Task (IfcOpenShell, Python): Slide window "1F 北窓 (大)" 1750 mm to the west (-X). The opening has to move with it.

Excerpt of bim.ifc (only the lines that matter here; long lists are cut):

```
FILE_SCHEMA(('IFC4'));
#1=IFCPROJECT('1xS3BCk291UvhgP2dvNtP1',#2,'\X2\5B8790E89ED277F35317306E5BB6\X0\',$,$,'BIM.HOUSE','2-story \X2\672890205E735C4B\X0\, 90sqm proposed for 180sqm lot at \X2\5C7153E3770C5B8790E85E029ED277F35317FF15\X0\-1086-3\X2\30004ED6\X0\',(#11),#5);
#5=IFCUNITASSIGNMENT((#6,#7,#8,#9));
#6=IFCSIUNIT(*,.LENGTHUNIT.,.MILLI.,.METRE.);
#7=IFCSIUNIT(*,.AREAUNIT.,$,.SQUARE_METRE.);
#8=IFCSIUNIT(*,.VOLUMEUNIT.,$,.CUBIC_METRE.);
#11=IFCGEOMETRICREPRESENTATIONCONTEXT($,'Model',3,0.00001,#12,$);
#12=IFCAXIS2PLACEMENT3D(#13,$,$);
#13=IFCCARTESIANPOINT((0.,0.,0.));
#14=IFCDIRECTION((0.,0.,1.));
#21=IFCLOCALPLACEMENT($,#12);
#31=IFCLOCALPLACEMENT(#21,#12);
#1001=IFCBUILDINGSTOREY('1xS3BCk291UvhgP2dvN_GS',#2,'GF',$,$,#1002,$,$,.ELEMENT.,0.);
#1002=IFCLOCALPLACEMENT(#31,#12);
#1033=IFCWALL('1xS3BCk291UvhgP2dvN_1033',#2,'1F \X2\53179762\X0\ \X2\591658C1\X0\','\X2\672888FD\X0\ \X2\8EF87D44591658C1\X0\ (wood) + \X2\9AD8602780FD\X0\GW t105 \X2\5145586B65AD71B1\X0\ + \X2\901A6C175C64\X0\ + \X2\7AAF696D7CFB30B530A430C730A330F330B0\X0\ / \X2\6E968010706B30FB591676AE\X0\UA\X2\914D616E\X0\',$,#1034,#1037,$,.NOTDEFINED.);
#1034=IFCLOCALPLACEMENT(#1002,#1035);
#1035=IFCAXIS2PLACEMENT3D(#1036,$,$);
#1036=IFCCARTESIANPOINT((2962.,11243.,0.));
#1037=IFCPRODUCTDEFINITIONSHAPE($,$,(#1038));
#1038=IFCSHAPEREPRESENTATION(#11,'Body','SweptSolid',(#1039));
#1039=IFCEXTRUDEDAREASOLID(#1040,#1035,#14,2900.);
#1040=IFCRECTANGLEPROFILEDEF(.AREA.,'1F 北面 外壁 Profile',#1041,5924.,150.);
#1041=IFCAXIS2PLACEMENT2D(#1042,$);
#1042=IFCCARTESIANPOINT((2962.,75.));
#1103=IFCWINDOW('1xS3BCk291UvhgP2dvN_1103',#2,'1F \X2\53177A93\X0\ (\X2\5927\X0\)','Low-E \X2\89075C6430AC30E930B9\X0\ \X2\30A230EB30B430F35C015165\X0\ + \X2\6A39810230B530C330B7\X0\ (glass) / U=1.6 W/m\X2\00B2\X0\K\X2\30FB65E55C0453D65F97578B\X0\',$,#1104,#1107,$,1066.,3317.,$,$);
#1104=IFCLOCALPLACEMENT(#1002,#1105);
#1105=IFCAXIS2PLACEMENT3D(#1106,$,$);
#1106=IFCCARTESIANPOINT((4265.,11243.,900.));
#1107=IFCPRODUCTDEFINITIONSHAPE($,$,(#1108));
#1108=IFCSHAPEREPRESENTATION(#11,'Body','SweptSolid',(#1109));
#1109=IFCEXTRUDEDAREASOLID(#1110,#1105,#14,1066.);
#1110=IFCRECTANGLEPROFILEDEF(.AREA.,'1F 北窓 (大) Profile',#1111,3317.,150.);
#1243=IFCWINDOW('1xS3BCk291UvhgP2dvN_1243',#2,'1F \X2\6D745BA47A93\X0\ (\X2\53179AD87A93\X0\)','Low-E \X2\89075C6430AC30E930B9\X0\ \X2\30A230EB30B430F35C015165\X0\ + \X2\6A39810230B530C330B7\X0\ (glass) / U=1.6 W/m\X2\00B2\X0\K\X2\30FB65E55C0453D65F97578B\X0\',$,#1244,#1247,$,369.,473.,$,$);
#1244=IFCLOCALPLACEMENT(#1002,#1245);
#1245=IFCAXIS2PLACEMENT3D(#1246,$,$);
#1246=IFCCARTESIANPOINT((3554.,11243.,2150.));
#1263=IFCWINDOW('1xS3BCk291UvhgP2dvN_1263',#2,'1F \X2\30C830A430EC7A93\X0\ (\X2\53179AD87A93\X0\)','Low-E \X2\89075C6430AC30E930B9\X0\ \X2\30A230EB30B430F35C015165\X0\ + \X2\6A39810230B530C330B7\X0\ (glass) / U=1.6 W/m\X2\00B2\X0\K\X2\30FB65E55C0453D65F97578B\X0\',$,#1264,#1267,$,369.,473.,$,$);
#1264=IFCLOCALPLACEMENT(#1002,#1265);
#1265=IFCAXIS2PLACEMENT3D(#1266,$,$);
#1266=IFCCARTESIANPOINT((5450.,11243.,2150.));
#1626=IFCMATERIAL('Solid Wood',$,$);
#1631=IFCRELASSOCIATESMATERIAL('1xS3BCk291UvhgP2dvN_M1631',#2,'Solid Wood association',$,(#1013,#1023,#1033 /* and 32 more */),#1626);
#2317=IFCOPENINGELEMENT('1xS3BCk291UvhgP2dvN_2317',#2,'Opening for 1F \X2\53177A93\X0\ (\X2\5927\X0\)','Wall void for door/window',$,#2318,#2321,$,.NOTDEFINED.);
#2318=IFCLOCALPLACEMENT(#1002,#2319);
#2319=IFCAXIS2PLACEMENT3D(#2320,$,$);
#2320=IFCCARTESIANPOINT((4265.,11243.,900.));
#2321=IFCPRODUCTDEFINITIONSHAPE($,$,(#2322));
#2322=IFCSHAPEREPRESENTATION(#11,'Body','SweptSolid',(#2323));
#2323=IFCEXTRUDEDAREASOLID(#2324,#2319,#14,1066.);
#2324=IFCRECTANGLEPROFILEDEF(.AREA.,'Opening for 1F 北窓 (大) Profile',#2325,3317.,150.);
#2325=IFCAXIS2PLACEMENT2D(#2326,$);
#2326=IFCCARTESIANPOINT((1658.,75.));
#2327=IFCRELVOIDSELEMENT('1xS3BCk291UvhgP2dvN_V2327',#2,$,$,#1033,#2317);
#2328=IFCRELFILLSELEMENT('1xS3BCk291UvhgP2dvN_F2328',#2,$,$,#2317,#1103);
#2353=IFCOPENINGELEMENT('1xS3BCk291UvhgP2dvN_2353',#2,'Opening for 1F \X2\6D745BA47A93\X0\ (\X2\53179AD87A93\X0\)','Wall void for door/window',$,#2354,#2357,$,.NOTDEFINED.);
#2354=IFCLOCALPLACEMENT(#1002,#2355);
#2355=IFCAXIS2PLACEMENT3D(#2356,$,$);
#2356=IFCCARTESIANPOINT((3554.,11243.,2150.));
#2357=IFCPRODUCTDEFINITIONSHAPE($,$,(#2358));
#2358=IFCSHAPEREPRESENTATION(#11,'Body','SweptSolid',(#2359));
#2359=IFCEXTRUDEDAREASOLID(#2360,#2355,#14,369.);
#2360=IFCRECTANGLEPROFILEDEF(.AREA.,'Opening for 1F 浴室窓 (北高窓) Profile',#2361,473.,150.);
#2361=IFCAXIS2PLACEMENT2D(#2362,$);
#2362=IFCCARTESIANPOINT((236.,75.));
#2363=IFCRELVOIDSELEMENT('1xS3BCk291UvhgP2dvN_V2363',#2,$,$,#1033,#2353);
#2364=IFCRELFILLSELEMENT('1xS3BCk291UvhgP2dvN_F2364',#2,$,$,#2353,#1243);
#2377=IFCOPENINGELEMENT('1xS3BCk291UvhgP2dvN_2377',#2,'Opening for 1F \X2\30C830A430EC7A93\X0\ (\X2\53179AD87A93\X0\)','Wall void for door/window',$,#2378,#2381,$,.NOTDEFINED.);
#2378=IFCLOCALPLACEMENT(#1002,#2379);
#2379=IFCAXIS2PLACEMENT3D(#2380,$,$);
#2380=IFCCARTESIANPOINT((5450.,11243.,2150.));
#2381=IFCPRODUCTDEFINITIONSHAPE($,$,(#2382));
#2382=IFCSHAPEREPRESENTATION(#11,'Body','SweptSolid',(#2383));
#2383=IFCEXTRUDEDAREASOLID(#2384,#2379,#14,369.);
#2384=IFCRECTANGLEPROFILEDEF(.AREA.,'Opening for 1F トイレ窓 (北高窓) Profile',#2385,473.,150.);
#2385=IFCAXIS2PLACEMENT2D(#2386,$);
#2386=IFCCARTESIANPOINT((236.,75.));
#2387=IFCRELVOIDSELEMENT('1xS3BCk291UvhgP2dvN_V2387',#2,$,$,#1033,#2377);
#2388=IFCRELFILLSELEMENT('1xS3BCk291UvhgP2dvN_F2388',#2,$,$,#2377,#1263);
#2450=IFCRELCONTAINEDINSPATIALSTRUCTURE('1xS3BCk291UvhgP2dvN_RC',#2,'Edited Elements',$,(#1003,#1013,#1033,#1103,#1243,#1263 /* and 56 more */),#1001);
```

```python
import ifcopenshell
import ifcopenshell.api.geometry
import ifcopenshell.util.placement
import ifcopenshell.util.unit

model = ifcopenshell.open("bim.ifc")
unit_scale = ifcopenshell.util.unit.calculate_unit_scale(model)

window = model.by_guid("1xS3BCk291UvhgP2dvN_1103")
opening = window.FillsVoids[0].RelatingOpeningElement
wall = opening.VoidsElements[0].RelatingBuildingElement

wall_matrix = ifcopenshell.util.placement.get_local_placement(wall.ObjectPlacement)
shift = wall_matrix[:3, 0] * -1.75 / unit_scale
before = ifcopenshell.util.placement.get_local_placement(window.ObjectPlacement)[:3, 3].copy()

# The window is not placed relative to its opening, so move both.
for product in (opening, window):
    matrix = ifcopenshell.util.placement.get_local_placement(product.ObjectPlacement)
    matrix[:3, 3] += shift
    ifcopenshell.api.geometry.edit_object_placement(model, product=product, matrix=matrix, is_si=False)

after = ifcopenshell.util.placement.get_local_placement(window.ObjectPlacement)[:3, 3]
print("window moved by", (after - before).round(3) + 0.0)

model.write("bim_updated.ifc")
```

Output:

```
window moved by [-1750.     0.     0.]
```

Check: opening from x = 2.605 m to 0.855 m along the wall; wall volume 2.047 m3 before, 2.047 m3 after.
